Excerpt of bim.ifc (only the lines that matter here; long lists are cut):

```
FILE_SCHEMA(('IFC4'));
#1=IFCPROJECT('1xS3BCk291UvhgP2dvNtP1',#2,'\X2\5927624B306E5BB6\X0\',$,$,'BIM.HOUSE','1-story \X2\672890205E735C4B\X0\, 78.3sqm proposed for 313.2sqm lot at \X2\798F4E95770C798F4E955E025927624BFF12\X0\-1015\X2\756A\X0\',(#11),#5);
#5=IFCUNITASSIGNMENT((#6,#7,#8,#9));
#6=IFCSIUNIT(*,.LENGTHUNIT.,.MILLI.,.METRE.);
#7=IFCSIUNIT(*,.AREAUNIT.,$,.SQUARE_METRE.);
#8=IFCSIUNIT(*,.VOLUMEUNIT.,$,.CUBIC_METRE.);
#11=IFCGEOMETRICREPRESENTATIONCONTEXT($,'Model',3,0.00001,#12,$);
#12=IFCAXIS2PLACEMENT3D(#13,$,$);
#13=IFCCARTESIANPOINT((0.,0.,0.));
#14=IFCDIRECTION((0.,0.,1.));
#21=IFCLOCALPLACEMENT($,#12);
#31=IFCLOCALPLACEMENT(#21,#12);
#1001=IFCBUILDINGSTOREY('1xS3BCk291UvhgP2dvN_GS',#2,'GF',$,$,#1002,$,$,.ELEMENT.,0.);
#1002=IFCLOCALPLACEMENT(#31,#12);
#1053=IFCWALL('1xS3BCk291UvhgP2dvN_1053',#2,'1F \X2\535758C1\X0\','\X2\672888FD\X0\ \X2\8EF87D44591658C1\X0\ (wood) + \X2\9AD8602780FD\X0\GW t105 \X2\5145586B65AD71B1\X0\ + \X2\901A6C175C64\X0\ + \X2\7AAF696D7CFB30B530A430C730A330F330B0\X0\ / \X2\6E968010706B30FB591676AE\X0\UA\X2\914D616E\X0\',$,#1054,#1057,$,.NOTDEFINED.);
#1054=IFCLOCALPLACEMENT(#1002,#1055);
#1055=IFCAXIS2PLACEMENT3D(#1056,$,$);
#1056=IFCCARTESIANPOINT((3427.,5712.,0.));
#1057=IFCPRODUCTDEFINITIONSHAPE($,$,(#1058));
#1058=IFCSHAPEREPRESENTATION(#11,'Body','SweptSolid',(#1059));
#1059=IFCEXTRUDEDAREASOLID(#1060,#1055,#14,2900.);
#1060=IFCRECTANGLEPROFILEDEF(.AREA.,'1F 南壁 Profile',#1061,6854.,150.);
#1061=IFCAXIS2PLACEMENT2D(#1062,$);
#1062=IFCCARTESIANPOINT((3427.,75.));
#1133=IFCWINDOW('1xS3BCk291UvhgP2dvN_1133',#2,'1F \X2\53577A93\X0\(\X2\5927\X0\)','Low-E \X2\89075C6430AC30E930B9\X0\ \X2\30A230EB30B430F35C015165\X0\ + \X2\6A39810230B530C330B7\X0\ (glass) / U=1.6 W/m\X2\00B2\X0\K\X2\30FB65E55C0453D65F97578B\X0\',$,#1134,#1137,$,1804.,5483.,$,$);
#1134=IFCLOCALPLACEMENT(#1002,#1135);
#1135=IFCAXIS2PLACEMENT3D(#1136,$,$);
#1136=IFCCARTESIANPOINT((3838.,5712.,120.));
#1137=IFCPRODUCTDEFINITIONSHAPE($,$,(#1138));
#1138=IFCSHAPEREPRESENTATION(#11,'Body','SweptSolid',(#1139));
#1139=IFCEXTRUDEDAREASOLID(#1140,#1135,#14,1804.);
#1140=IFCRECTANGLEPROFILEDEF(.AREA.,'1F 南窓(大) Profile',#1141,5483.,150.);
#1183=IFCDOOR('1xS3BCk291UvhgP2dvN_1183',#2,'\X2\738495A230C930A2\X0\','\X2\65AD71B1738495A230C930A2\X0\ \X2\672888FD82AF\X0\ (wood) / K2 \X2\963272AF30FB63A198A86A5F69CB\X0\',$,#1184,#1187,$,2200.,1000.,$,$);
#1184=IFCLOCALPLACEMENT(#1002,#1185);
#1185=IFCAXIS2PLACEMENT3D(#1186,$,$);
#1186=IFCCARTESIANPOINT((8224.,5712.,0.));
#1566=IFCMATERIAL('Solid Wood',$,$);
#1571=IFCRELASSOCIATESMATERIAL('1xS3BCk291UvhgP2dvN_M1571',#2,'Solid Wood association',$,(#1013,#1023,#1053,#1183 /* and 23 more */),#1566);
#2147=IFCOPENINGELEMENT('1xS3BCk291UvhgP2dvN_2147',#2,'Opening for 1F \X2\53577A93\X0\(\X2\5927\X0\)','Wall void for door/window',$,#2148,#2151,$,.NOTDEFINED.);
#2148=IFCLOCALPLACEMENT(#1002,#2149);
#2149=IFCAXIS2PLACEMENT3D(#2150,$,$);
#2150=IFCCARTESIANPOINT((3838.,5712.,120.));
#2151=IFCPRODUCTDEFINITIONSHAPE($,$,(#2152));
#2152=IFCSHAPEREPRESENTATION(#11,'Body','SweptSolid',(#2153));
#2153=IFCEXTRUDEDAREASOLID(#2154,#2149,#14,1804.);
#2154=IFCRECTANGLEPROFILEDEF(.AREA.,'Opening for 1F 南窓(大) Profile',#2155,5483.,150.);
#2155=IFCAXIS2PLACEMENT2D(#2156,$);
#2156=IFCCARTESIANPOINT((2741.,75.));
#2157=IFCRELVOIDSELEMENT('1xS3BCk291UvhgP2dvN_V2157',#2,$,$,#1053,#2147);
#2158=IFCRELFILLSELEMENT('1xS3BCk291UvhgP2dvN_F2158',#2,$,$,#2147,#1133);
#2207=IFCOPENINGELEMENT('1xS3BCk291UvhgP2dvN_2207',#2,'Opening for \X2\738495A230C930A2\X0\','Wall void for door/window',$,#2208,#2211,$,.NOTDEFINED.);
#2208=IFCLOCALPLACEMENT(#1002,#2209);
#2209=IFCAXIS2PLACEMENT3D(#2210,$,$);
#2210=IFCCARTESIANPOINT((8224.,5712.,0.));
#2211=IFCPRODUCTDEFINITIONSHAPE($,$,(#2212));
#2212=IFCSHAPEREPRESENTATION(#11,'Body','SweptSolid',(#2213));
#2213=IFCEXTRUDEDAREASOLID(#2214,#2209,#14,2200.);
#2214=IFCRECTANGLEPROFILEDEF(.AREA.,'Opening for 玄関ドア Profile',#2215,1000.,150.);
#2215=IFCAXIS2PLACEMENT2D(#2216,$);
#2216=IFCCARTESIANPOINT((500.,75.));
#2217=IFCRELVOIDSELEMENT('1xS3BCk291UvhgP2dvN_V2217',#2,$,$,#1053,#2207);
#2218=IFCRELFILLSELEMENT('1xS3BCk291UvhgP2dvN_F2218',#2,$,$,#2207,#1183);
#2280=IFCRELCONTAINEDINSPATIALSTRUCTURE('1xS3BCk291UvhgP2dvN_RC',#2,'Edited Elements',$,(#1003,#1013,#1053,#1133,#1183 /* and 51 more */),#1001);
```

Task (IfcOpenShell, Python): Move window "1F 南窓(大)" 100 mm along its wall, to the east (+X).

```python
import ifcopenshell
import ifcopenshell.api.geometry
import ifcopenshell.util.placement
import ifcopenshell.util.unit

model = ifcopenshell.open("bim.ifc")
unit_scale = ifcopenshell.util.unit.calculate_unit_scale(model)

window = model.by_guid("1xS3BCk291UvhgP2dvN_1133")
opening = window.FillsVoids[0].RelatingOpeningElement
wall = opening.VoidsElements[0].RelatingBuildingElement

wall_matrix = ifcopenshell.util.placement.get_local_placement(wall.ObjectPlacement)
shift = wall_matrix[:3, 0] * 0.1 / unit_scale
before = ifcopenshell.util.placement.get_local_placement(window.ObjectPlacement)[:3, 3].copy()

# The window is not placed relative to its opening, so move both.
for product in (opening, window):
    matrix = ifcopenshell.util.placement.get_local_placement(product.ObjectPlacement)
    matrix[:3, 3] += shift
    ifcopenshell.api.geometry.edit_object_placement(model, product=product, matrix=matrix, is_si=False)

after = ifcopenshell.util.placement.get_local_placement(window.ObjectPlacement)[:3, 3]
print("window moved by", (after - before).round(3) + 0.0)

model.write("bim_v2.ifc")
```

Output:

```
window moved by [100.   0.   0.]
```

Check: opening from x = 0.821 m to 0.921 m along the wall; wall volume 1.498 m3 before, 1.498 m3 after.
